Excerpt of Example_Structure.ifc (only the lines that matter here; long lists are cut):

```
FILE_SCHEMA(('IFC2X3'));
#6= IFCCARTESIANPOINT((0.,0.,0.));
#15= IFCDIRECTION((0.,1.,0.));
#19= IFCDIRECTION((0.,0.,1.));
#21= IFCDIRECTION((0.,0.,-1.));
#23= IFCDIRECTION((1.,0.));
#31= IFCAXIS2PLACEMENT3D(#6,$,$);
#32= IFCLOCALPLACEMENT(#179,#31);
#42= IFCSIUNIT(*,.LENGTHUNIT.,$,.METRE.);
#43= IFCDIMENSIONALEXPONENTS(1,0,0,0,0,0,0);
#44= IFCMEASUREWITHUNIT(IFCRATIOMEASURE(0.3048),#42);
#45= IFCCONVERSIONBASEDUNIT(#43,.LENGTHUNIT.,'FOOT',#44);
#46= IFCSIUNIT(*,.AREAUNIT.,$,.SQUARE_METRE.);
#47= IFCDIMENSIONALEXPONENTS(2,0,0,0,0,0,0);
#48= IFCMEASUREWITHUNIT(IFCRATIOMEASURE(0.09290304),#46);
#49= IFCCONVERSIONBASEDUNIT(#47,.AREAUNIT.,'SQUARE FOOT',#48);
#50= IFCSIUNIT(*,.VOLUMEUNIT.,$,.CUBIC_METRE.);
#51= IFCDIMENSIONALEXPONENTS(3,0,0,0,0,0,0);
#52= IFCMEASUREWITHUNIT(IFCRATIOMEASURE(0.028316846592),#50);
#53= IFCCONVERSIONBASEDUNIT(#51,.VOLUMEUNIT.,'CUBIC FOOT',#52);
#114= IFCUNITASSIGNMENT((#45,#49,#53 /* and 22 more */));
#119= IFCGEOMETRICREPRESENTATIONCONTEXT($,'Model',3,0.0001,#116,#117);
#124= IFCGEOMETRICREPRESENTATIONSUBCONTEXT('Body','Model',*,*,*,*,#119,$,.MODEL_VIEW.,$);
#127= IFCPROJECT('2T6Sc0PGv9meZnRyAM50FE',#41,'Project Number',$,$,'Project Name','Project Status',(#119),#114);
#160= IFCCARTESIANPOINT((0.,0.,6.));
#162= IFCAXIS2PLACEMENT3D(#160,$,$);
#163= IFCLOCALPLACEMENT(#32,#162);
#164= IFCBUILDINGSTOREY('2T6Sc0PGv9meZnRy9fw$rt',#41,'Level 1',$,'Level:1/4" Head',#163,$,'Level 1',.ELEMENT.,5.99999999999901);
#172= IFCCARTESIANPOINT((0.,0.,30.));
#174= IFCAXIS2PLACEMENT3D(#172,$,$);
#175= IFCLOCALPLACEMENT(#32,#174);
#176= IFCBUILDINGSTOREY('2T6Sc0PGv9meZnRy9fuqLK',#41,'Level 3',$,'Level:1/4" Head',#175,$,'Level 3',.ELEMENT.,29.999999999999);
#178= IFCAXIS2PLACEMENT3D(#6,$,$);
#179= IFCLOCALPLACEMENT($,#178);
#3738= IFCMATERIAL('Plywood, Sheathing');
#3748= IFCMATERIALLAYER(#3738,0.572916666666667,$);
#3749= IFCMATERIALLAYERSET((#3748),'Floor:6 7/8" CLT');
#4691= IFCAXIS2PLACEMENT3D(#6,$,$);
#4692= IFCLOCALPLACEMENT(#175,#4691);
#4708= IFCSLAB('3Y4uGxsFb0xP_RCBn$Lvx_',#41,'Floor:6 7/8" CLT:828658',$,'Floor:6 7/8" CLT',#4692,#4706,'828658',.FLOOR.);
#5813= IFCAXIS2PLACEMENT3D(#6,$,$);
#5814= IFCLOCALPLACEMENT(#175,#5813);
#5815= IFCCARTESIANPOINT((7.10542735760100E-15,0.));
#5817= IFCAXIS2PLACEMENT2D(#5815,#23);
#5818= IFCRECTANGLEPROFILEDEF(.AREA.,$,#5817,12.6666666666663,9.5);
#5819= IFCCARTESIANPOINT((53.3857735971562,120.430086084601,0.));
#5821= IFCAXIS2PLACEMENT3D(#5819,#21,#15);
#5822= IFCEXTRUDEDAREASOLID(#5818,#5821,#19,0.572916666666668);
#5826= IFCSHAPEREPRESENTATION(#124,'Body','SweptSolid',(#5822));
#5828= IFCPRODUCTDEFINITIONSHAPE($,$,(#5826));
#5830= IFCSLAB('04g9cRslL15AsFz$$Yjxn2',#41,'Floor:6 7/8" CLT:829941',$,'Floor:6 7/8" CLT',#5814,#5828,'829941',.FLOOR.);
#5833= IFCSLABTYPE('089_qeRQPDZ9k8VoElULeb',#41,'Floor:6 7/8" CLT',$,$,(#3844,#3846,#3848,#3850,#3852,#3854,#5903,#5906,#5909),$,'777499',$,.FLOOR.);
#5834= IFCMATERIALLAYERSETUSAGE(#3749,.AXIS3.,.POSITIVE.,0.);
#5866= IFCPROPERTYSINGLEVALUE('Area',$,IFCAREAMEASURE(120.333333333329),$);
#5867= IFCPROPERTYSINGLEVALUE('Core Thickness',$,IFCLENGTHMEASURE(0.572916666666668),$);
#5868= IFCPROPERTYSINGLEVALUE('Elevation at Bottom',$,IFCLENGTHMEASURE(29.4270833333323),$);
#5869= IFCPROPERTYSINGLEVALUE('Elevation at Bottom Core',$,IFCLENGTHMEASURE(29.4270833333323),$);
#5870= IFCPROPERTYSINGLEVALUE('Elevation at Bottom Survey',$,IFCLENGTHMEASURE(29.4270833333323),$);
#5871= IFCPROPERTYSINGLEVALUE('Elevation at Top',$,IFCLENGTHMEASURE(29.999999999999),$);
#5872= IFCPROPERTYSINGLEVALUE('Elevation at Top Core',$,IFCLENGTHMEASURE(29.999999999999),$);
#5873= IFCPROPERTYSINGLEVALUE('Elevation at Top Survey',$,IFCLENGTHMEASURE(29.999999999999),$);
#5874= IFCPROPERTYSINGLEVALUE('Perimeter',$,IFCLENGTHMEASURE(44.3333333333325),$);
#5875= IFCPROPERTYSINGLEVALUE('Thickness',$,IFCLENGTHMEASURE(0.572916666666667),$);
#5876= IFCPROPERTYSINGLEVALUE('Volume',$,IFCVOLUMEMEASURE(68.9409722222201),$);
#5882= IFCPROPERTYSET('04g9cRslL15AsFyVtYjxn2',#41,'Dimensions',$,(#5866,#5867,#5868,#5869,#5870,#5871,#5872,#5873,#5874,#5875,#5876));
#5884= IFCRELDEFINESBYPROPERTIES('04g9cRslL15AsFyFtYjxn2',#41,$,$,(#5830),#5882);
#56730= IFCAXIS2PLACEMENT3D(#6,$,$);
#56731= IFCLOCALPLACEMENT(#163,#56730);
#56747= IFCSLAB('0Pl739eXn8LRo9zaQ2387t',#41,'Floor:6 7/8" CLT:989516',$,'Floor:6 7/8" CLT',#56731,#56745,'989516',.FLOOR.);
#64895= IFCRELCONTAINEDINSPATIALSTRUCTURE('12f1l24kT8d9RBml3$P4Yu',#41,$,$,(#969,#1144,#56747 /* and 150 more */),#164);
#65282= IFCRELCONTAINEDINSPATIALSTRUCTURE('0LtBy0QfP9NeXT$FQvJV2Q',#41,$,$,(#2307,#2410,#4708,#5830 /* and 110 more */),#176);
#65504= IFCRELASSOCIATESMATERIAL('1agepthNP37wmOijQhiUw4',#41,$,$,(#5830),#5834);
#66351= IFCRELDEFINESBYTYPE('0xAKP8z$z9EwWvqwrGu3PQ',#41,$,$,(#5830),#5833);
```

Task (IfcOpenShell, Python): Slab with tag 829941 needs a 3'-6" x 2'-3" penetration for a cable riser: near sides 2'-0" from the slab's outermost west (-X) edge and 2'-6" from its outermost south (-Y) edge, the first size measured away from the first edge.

```python
import numpy as np
import ifcopenshell
import ifcopenshell.api.feature
import ifcopenshell.api.geometry
import ifcopenshell.api.pset
import ifcopenshell.api.root
import ifcopenshell.geom
import ifcopenshell.util.element
import ifcopenshell.util.placement
import ifcopenshell.util.representation
import ifcopenshell.util.shape
import ifcopenshell.util.unit

model = ifcopenshell.open("Example_Structure.ifc")
unit_scale = ifcopenshell.util.unit.calculate_unit_scale(model)
area_scale = ifcopenshell.util.unit.calculate_unit_scale(model, "AREAUNIT")
volume_scale = ifcopenshell.util.unit.calculate_unit_scale(model, "VOLUMEUNIT")
settings = ifcopenshell.geom.settings()


def volume(element):
    """Net volume in cubic metres, openings subtracted."""
    shape = ifcopenshell.geom.create_shape(settings, element)
    return ifcopenshell.util.shape.get_volume(shape.geometry)


slab = model.by_guid("04g9cRslL15AsFz$$Yjxn2")
before = volume(slab)

# Extent in the slab's own axes, in metres. The edges named are its -X and -Y sides.
slab_shape = ifcopenshell.geom.create_shape(settings, slab)
vertices = ifcopenshell.util.shape.get_vertices(slab_shape.geometry)
x_min, y_min, bottom = vertices.min(axis=0)
top = vertices[:, 2].max()

opening = ifcopenshell.api.root.create_entity(model, ifc_class="IfcOpeningElement", name="Cable riser opening")
context = ifcopenshell.util.representation.get_context(model, "Model", "Body", "MODEL_VIEW")
width, depth = 1.0668, 0.6858
outline = [(0.0, 0.0), (width, 0.0), (width, depth), (0.0, depth), (0.0, 0.0)]
# Overshoot both faces by 50 mm so the cut is clean.
shape = ifcopenshell.api.geometry.add_slab_representation(
    model, context=context, depth=top - bottom + 0.1, polyline=outline
)
ifcopenshell.api.geometry.assign_representation(model, product=opening, representation=shape)

matrix = ifcopenshell.util.placement.get_local_placement(slab.ObjectPlacement)
matrix[:, 3] = matrix @ np.append(np.array([x_min + 0.6096, y_min + 0.762, bottom - 0.05]) / unit_scale, 1.0)
ifcopenshell.api.geometry.edit_object_placement(model, product=opening, matrix=matrix, is_si=False)
ifcopenshell.api.feature.add_feature(model, feature=opening, element=slab)

after = volume(slab)

# Update the slab's stored quantities.
pset = model.by_id(ifcopenshell.util.element.get_pset(slab, "Dimensions", should_inherit=False)["id"])
ifcopenshell.api.pset.edit_pset(model, pset=pset, properties={
    "Area": model.create_entity("IfcAreaMeasure", after / (top - bottom) / area_scale),
    "Volume": model.create_entity("IfcVolumeMeasure", after / volume_scale),
})

print(f"slab volume {before:.3f} -> {after:.3f} m3")

model.write("Example_Structure_v2.ifc")
```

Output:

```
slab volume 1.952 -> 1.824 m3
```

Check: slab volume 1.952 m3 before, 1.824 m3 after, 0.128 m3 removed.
